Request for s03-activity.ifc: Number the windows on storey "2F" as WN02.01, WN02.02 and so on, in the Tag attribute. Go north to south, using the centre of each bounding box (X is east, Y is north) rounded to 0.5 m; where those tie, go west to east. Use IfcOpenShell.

First a look at what the model holds.

```python
import ifcopenshell
import ifcopenshell.util.element
import ifcopenshell.util.placement

model = ifcopenshell.open("s03-activity.ifc")
print(model.schema)
storey = next(s for s in model.by_type("IfcBuildingStorey") if s.Name == "2F")
windows = [e for e in ifcopenshell.util.element.get_decomposition(storey) if e.is_a("IfcWindow")]
for e in sorted(windows, key=lambda e: e.id()):
    origin = ifcopenshell.util.placement.get_local_placement(e.ObjectPlacement)[:3, 3]
    print(e.id(), e.Tag, e.Name, origin.round(2) + 0.0, sep=" | ")
```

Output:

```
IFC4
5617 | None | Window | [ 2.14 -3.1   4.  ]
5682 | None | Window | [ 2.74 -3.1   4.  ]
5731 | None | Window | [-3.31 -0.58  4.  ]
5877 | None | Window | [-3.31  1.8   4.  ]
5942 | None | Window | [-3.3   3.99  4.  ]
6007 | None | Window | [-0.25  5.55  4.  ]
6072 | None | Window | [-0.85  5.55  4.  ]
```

```python
import ifcopenshell
import ifcopenshell.geom
import ifcopenshell.util.element
import ifcopenshell.util.shape

model = ifcopenshell.open("s03-activity.ifc")
settings = ifcopenshell.geom.settings()
settings.set("use-world-coords", True)


def centre(element):
    shape = ifcopenshell.geom.create_shape(settings, element)
    return ifcopenshell.util.shape.get_bbox_centroid(shape.geometry)


storey = next(s for s in model.by_type("IfcBuildingStorey") if s.Name == "2F")
windows = [e for e in ifcopenshell.util.element.get_decomposition(storey) if e.is_a("IfcWindow")]

# Insertion points can sit at a corner or the storey origin, so sort by the geometry (in metres).
centres = {e: centre(e) for e in windows}
windows.sort(key=lambda e: (-round(centres[e][1] / 0.5), centres[e][0]))

for i, e in enumerate(windows, start=1):
    number = f"WN02.{i:02d}"
    e.Tag = number
    print(e.id(), number)

model.write("s03-activity-out.ifc")
```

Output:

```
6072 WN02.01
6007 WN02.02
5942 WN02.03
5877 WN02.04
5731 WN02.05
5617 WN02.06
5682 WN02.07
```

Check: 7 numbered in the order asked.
